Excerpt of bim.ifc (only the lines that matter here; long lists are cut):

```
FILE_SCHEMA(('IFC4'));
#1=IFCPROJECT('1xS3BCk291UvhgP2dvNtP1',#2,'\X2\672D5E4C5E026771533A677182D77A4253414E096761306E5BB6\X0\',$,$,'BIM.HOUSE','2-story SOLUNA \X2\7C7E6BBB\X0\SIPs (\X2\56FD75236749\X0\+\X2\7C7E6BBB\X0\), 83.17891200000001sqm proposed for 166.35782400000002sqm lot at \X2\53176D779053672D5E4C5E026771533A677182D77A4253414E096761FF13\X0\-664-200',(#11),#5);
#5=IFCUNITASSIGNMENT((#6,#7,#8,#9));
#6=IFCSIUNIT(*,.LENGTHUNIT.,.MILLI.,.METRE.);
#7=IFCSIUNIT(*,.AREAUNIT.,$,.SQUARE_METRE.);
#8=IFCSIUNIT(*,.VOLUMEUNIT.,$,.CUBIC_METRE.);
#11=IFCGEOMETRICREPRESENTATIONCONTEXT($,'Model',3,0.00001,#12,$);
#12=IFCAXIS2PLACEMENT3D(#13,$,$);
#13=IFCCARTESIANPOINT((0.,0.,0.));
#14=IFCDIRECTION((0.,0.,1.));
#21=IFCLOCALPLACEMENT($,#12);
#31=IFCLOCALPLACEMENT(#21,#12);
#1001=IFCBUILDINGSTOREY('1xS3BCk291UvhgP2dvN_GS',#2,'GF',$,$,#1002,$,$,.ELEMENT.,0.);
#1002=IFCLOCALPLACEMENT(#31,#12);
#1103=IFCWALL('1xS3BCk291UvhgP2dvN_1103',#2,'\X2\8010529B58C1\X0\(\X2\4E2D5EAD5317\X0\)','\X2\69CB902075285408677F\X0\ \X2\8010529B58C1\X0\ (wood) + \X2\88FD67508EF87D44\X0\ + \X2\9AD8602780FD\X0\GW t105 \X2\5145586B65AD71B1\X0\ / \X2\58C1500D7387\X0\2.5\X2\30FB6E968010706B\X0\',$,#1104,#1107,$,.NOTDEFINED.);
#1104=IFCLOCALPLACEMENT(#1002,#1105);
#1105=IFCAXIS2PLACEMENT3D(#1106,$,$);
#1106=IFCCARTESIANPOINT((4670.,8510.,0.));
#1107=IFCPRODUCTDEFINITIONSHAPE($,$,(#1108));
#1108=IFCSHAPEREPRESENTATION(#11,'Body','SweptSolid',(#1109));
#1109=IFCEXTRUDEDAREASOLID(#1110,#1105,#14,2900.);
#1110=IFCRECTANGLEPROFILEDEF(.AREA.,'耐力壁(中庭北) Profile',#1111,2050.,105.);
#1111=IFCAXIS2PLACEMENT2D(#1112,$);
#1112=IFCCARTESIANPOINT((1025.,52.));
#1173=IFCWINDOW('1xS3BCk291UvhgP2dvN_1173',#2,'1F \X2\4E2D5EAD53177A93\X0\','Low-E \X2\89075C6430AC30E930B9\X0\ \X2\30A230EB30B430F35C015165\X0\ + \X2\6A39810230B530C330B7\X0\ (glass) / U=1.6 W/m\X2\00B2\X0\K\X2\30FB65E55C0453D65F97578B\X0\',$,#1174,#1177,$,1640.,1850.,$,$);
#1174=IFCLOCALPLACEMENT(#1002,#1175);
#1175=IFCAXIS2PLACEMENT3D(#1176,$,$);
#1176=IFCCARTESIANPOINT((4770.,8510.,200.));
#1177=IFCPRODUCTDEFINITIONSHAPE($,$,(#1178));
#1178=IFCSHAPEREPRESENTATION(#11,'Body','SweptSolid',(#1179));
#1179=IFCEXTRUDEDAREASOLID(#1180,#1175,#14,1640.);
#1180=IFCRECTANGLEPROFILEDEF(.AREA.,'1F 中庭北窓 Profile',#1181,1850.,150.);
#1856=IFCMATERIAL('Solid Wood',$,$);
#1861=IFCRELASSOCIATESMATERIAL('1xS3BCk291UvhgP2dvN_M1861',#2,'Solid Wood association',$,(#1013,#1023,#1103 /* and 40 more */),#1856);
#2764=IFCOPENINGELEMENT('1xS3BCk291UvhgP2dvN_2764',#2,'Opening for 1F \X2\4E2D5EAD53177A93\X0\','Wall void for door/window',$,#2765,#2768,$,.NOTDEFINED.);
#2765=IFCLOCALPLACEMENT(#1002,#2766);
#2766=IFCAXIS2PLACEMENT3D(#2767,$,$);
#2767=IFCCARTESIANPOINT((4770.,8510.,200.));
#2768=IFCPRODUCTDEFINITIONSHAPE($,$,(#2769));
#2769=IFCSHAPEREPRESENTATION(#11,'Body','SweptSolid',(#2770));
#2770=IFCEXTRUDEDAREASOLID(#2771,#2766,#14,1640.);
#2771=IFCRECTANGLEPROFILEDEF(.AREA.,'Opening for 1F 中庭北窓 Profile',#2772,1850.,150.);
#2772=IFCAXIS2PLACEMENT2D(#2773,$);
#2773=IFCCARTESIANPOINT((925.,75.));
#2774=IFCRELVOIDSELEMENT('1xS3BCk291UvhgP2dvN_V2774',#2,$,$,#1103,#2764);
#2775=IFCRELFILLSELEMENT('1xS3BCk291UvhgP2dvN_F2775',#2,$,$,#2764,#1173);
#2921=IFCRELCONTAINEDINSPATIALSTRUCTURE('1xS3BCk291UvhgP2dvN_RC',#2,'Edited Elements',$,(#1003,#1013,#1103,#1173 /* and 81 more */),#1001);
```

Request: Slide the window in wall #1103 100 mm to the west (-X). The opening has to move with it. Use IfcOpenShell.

```python
import ifcopenshell
import ifcopenshell.api.geometry
import ifcopenshell.util.placement

model = ifcopenshell.open("bim.ifc")

window = model.by_guid("1xS3BCk291UvhgP2dvN_1173")
opening = window.FillsVoids[0].RelatingOpeningElement
wall = opening.VoidsElements[0].RelatingBuildingElement

wall_matrix = ifcopenshell.util.placement.get_local_placement(wall.ObjectPlacement)
shift = wall_matrix[:3, 0] * -100.0
before = ifcopenshell.util.placement.get_local_placement(window.ObjectPlacement)[:3, 3].copy()

# The window is not placed relative to its opening, so move both.
for product in (opening, window):
    matrix = ifcopenshell.util.placement.get_local_placement(product.ObjectPlacement)
    matrix[:3, 3] += shift
    ifcopenshell.api.geometry.edit_object_placement(model, product=product, matrix=matrix, is_si=False)

after = ifcopenshell.util.placement.get_local_placement(window.ObjectPlacement)[:3, 3]
print("window moved by", (after - before).round(3) + 0.0)

model.write("bim_updated.ifc")
```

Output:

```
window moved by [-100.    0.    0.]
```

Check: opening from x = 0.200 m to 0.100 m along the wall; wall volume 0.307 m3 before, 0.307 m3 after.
